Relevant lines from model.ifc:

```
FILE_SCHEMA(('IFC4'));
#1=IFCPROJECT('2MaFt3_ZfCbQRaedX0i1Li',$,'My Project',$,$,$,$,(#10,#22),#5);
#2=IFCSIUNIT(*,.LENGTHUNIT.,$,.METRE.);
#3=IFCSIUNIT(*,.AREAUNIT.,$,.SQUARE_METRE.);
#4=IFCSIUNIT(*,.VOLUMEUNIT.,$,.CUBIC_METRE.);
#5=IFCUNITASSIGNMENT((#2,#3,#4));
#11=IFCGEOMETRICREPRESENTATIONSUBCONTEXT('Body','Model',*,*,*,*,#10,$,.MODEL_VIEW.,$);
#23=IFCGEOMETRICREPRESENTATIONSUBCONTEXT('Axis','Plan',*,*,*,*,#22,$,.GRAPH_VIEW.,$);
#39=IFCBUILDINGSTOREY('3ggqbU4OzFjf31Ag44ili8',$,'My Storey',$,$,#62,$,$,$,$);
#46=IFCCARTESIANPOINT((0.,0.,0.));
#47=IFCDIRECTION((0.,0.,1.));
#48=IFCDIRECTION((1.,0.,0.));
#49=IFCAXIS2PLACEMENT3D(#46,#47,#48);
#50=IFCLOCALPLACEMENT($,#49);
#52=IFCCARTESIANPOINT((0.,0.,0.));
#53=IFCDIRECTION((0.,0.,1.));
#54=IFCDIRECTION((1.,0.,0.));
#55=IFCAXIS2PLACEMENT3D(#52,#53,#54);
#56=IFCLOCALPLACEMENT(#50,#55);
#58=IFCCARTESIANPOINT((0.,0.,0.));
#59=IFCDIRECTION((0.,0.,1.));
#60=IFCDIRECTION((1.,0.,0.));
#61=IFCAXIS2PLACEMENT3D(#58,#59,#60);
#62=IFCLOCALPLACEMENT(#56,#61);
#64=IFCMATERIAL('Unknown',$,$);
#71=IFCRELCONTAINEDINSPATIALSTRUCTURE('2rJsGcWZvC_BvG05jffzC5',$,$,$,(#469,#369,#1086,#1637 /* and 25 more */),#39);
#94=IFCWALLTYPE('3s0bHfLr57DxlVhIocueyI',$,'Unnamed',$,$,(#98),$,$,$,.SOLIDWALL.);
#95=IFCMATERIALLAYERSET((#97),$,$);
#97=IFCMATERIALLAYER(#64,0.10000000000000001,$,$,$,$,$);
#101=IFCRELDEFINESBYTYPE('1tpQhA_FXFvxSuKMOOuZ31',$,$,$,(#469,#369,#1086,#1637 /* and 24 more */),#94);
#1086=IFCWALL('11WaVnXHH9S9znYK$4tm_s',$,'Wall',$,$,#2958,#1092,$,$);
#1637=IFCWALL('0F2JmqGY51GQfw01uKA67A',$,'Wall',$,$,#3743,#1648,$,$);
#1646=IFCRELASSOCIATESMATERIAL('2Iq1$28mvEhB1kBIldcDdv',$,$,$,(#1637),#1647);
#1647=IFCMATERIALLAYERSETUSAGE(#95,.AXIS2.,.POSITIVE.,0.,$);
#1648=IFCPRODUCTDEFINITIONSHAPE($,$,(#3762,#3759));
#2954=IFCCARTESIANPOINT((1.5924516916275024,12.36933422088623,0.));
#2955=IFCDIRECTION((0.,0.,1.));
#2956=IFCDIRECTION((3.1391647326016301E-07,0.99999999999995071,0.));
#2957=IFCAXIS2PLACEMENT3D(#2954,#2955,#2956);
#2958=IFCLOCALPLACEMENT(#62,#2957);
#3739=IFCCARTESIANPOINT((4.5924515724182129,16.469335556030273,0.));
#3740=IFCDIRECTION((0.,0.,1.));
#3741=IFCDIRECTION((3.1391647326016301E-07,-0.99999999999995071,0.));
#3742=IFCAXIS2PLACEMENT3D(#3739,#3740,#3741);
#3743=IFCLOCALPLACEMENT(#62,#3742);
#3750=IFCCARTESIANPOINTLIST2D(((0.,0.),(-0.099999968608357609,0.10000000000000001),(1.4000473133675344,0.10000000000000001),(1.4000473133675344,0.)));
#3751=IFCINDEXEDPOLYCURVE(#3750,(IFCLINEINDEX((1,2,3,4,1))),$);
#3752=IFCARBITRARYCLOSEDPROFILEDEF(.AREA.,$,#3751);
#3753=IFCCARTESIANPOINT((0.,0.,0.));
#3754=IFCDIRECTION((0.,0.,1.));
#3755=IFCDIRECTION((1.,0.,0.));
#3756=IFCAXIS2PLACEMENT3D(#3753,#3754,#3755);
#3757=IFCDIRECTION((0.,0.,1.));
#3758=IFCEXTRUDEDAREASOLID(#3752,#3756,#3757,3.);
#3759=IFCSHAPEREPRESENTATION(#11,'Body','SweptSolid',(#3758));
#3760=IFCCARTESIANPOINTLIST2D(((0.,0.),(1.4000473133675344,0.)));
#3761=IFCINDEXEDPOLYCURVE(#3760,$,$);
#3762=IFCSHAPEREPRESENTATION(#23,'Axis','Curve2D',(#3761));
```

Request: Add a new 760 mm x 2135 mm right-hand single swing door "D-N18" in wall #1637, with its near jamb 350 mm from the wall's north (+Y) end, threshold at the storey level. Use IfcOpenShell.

```python
import numpy as np
import ifcopenshell
import ifcopenshell.api.feature
import ifcopenshell.api.geometry
import ifcopenshell.api.root
import ifcopenshell.api.spatial
import ifcopenshell.geom
import ifcopenshell.util.element
import ifcopenshell.util.placement
import ifcopenshell.util.representation
import ifcopenshell.util.shape
import ifcopenshell.util.unit

model = ifcopenshell.open("model.ifc")
unit_scale = ifcopenshell.util.unit.calculate_unit_scale(model)
settings = ifcopenshell.geom.settings()


def volume(element):
    """Net volume in cubic metres, openings subtracted."""
    shape = ifcopenshell.geom.create_shape(settings, element)
    return ifcopenshell.util.shape.get_volume(shape.geometry)


wall = model.by_guid("0F2JmqGY51GQfw01uKA67A")
storey = ifcopenshell.util.element.get_container(wall, ifc_class="IfcBuildingStorey")
context = ifcopenshell.util.representation.get_context(model, "Model", "Body", "MODEL_VIEW")
before = volume(wall)

width, height, from_end, sill = 0.76, 2.135, 0.35, 0.0  # metres

# The wall runs along its own X axis, and the end named is its -X end.
wall_shape = ifcopenshell.geom.create_shape(settings, wall)
x, y, z = ifcopenshell.util.shape.get_vertices(wall_shape.geometry).T
start = x.min() + from_end
face, thickness = float(y.min()), float(y.max() - y.min())
wall_matrix = ifcopenshell.util.placement.get_local_placement(wall.ObjectPlacement)
level = ifcopenshell.util.placement.get_local_placement(storey.ObjectPlacement)[2, 3]


def in_wall(x, y):
    """Placement at x, y metres in the wall's axes, at sill height."""
    matrix = wall_matrix.copy()
    matrix[:, 3] = wall_matrix @ np.array([x / unit_scale, y / unit_scale, 0.0, 1.0])
    matrix[2, 3] = level + sill / unit_scale
    return matrix


# Opening: a box that overshoots both wall faces by 50 mm.
opening = ifcopenshell.api.root.create_entity(model, ifc_class="IfcOpeningElement", predefined_type="OPENING")
box = ifcopenshell.api.geometry.add_wall_representation(
    model, context=context, length=width, height=height, thickness=thickness + 0.1
)
ifcopenshell.api.geometry.assign_representation(model, product=opening, representation=box)
ifcopenshell.api.geometry.edit_object_placement(model, product=opening, matrix=in_wall(start, face - 0.05), is_si=False)
ifcopenshell.api.feature.add_feature(model, feature=opening, element=wall)

door = ifcopenshell.api.root.create_entity(model, ifc_class="IfcDoor", name="D-N18", predefined_type="DOOR")
door.OverallWidth, door.OverallHeight = width / unit_scale, height / unit_scale
door.OperationType = "SINGLE_SWING_RIGHT"
body = ifcopenshell.api.geometry.add_door_representation(
    model,
    context=context,
    overall_width=door.OverallWidth,
    overall_height=door.OverallHeight,
    operation_type="SINGLE_SWING_RIGHT",
    lining_properties={"LiningDepth": thickness / unit_scale, "ThresholdDepth": thickness / unit_scale},
)
ifcopenshell.api.geometry.assign_representation(model, product=door, representation=body)
ifcopenshell.api.spatial.assign_container(model, products=[door], relating_structure=storey)
ifcopenshell.api.feature.add_filling(model, opening=opening, element=door)

# The lining spans the wall, so the door starts at the wall face.
ifcopenshell.api.geometry.edit_object_placement(model, product=door, matrix=in_wall(start, face), is_si=False)

after = volume(wall)

print(f"wall volume {before:.3f} -> {after:.3f} m3")

model.write("model-out.ifc")
```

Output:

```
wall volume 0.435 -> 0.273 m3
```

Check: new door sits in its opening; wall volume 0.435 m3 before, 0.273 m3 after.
